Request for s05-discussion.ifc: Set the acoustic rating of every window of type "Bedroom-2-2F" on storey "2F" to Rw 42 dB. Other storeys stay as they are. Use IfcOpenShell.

First a look at what the model holds.

```python
import ifcopenshell
import ifcopenshell.util.element

model = ifcopenshell.open("s05-discussion.ifc")
print(model.schema)
storey = next(s for s in model.by_type("IfcBuildingStorey") if s.Name == "2F")
windows = [e for e in ifcopenshell.util.element.get_decomposition(storey) if e.is_a("IfcWindow")]
seen = {}
for e in windows:
    element_type = ifcopenshell.util.element.get_type(e)
    key = (element_type.Name if element_type != e and element_type else None, ifcopenshell.util.element.get_pset(e, "Pset_WindowCommon", "AcousticRating"))
    seen[key] = seen.get(key, 0) + 1
for (name, value), count in sorted(seen.items(), key=str):
    print(count, "x", name, "|", value)
```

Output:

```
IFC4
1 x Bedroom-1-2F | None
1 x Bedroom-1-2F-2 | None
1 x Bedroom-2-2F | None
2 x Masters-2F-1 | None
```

```python
import ifcopenshell
import ifcopenshell.api.pset
import ifcopenshell.util.element

model = ifcopenshell.open("s05-discussion.ifc")

storey = next(s for s in model.by_type("IfcBuildingStorey") if s.Name == "2F")
windows = [e for e in ifcopenshell.util.element.get_decomposition(storey) if e.is_a("IfcWindow")]

count = 0
for e in windows:
    element_type = ifcopenshell.util.element.get_type(e)
    if element_type in (None, e) or element_type.Name != "Bedroom-2-2F":
        continue
    # add_pset returns the element's existing set when there is one.
    pset = ifcopenshell.api.pset.add_pset(model, product=e, name="Pset_WindowCommon")
    ifcopenshell.api.pset.edit_pset(model, pset=pset, properties={"AcousticRating": "Rw 42 dB"})
    count += 1

print(count, "windows updated")

model.write("s05-discussion_edited.ifc")
```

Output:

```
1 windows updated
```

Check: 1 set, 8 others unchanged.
